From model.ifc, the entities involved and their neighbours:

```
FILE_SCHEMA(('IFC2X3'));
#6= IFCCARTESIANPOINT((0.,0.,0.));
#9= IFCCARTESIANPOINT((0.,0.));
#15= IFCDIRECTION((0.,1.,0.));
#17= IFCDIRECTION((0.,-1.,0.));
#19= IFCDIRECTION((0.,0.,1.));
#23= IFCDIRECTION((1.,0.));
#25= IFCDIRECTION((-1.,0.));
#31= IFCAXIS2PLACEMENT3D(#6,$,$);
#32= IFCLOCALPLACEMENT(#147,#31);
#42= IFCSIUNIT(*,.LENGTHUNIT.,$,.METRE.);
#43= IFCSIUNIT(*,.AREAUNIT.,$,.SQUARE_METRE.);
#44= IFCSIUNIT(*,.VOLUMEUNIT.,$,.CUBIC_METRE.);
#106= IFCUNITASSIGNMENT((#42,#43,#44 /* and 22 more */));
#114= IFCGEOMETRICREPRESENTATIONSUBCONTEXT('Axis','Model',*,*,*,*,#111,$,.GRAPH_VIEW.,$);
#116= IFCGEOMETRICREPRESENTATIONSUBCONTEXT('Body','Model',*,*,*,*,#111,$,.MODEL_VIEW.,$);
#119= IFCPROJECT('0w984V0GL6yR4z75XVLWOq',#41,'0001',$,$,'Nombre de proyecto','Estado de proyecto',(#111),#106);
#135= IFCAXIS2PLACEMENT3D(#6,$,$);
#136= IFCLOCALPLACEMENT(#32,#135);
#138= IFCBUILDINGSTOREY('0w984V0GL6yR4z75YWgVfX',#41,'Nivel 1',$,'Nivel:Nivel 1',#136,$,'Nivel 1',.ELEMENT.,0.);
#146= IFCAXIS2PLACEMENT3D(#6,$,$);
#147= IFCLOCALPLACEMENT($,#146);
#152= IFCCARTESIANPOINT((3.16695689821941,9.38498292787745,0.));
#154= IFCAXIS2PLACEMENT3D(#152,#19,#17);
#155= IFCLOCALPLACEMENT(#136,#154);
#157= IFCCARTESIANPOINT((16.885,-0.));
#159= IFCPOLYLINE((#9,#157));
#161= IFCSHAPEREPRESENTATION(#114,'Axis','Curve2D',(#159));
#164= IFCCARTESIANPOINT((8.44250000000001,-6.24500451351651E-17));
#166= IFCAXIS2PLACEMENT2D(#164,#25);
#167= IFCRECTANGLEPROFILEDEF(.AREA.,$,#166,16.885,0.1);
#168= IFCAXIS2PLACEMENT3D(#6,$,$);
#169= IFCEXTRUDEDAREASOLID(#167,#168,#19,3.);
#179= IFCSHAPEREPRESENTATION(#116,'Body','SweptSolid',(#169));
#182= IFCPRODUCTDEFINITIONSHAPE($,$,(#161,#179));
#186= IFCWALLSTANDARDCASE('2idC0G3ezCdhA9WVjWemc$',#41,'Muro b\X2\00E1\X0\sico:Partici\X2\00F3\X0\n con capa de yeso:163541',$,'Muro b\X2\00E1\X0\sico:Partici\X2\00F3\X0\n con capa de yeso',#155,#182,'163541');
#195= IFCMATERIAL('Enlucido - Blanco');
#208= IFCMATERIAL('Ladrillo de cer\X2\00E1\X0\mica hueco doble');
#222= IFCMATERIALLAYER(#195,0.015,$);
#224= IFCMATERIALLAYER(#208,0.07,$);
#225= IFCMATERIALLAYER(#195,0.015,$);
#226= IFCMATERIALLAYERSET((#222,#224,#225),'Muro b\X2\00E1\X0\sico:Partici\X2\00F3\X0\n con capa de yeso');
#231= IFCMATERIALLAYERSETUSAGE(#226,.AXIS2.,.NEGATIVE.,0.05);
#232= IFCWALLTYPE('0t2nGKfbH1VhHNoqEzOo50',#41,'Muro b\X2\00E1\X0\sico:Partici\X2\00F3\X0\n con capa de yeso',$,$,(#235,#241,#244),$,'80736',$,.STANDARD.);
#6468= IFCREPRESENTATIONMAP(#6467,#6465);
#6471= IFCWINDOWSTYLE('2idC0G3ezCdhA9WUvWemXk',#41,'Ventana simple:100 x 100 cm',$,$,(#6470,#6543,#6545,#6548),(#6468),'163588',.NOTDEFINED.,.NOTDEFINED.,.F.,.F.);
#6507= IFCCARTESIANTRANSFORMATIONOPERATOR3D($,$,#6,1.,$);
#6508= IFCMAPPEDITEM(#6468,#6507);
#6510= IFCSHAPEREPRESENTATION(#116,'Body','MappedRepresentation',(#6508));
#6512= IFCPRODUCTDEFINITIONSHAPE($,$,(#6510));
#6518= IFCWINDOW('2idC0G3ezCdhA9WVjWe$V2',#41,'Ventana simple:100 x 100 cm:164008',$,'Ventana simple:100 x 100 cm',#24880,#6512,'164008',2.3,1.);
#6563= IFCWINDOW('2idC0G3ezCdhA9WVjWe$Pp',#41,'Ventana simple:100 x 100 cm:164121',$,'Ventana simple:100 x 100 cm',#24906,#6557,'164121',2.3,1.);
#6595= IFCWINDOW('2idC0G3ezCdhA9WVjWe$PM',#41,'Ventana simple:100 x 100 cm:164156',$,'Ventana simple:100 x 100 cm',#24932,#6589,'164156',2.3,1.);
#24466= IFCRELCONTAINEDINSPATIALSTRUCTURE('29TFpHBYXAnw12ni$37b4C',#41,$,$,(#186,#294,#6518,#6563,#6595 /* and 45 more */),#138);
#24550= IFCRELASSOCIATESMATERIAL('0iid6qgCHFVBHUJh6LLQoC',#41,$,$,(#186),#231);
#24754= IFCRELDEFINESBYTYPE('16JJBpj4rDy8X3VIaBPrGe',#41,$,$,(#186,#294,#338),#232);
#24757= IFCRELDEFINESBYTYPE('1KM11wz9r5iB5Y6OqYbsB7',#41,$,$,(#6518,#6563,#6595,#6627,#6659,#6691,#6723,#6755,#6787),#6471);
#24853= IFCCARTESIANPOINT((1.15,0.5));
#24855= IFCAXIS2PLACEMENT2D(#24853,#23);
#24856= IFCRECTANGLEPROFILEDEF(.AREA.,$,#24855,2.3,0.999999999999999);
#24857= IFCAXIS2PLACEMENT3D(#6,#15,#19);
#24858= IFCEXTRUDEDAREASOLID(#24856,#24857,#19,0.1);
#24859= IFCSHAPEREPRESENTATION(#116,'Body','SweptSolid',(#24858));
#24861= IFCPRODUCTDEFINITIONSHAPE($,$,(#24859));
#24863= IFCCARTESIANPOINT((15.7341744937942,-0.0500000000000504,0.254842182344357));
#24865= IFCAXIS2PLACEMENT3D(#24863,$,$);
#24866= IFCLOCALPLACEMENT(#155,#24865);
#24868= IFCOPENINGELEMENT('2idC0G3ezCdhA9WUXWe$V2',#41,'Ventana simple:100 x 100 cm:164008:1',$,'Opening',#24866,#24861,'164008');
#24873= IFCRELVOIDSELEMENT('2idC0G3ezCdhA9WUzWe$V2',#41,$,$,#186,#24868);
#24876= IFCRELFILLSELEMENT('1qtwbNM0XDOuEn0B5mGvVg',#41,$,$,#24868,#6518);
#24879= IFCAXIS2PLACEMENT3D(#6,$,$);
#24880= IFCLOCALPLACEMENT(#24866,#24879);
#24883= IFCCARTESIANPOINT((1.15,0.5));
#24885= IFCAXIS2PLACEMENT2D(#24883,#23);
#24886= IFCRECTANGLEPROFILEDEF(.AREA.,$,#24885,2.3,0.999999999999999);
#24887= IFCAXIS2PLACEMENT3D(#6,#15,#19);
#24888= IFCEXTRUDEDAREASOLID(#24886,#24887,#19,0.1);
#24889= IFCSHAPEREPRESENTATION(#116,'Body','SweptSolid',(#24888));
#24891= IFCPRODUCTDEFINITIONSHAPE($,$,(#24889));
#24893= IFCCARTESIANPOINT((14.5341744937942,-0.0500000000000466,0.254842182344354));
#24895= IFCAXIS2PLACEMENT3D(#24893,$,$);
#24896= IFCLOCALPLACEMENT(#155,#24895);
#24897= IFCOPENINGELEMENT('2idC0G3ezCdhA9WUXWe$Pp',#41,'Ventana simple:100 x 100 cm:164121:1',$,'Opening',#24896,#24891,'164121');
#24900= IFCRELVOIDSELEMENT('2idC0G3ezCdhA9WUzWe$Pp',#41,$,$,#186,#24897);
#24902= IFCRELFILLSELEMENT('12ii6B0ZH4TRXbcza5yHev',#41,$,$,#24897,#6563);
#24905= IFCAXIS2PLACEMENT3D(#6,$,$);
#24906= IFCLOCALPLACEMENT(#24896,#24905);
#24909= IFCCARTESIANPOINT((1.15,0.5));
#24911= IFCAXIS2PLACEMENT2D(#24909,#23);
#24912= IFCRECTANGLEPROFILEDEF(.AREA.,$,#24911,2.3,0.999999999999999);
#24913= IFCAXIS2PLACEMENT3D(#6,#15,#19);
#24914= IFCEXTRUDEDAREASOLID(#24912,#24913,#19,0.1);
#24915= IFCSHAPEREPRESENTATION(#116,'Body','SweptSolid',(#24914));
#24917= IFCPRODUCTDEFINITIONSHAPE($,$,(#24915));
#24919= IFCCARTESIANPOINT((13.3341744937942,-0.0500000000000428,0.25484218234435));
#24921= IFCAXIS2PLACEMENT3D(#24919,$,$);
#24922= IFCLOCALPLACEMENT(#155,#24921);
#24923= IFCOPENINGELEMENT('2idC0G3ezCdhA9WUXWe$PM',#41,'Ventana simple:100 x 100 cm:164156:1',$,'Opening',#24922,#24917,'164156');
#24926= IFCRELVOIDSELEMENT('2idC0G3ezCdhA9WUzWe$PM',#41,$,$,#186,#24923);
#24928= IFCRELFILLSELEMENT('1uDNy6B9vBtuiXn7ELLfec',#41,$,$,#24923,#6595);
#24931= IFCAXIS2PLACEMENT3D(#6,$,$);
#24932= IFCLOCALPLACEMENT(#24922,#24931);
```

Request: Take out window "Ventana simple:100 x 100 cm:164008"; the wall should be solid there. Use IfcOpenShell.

```python
import ifcopenshell
import ifcopenshell.api.feature
import ifcopenshell.api.root
import ifcopenshell.geom
import ifcopenshell.util.shape

model = ifcopenshell.open("model.ifc")
settings = ifcopenshell.geom.settings()


def volume(element):
    """Net volume in cubic metres, openings subtracted."""
    shape = ifcopenshell.geom.create_shape(settings, element)
    return ifcopenshell.util.shape.get_volume(shape.geometry)


window = model.by_id(6518)
opening = window.FillsVoids[0].RelatingOpeningElement
wall = opening.VoidsElements[0].RelatingBuildingElement
before = volume(wall)

ifcopenshell.api.root.remove_product(model, product=window)
ifcopenshell.api.feature.remove_feature(model, feature=opening)

after = volume(wall)

print(f"wall volume {before:.3f} -> {after:.3f} m3")

model.write("model_rev.ifc")
```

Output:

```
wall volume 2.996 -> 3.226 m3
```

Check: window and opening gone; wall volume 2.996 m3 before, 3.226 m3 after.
